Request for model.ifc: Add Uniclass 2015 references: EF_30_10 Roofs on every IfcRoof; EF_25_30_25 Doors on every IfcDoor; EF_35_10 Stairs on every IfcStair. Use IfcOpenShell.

First a look at what the model holds.

```python
import ifcopenshell

model = ifcopenshell.open("model.ifc")
print(model.schema)
print("classifications:", [c.Name for c in model.by_type("IfcClassification")])
for ifc_class in ("IfcDoor", "IfcRoof", "IfcStair", "IfcWall", "IfcWindow"):
    print(ifc_class, len(model.by_type(ifc_class)))
```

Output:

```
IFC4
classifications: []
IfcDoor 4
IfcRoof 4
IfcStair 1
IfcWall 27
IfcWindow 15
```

```python
import ifcopenshell
import ifcopenshell.api.classification

model = ifcopenshell.open("model.ifc")

system = ifcopenshell.api.classification.add_classification(model, classification="Uniclass 2015")

codes = {
    "IfcRoof": ("EF_30_10", "Roofs"),
    "IfcDoor": ("EF_25_30_25", "Doors"),
    "IfcStair": ("EF_35_10", "Stairs"),
}
for ifc_class, (code, name) in codes.items():
    products = model.by_type(ifc_class)
    ifcopenshell.api.classification.add_reference(
        model, products=products, classification=system, identification=code, name=name
    )
    print(code, len(products))

model.write("model_v2.ifc")
```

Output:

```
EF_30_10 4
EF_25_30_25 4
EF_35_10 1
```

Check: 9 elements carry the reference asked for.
